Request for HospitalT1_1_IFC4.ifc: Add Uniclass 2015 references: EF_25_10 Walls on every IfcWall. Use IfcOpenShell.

First a look at what the model holds.

```python
import ifcopenshell

model = ifcopenshell.open("HospitalT1_1_IFC4.ifc")
print(model.schema)
print("classifications:", [c.Name for c in model.by_type("IfcClassification")])
for ifc_class in ("IfcDoor", "IfcRoof", "IfcStair", "IfcWall", "IfcWindow"):
    print(ifc_class, len(model.by_type(ifc_class)))
```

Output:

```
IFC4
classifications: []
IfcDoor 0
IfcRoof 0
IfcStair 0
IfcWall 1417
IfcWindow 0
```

```python
import ifcopenshell
import ifcopenshell.api.classification

model = ifcopenshell.open("HospitalT1_1_IFC4.ifc")

system = ifcopenshell.api.classification.add_classification(model, classification="Uniclass 2015")

codes = {
    "IfcWall": ("EF_25_10", "Walls"),
}
for ifc_class, (code, name) in codes.items():
    products = model.by_type(ifc_class)
    ifcopenshell.api.classification.add_reference(
        model, products=products, classification=system, identification=code, name=name
    )
    print(code, len(products))

model.write("HospitalT1_1_IFC4_rev.ifc")
```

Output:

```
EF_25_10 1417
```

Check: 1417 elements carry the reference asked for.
